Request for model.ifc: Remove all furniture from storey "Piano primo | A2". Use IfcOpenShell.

First a look at what the model holds.

```python
import ifcopenshell
import ifcopenshell.util.element

model = ifcopenshell.open("model.ifc")
print(model.schema)
storey = next(s for s in model.by_type("IfcBuildingStorey") if s.Name == "Piano primo | A2")
furniture = [e for e in ifcopenshell.util.element.get_decomposition(storey) if e.is_a("IfcFurnishingElement")]
seen = {}
for e in furniture:
    element_type = ifcopenshell.util.element.get_type(e)
    name = element_type.Name if element_type not in (None, e) else None
    seen[name] = seen.get(name, 0) + 1
for name, count in sorted(seen.items(), key=str):
    print(count, "x", name)
```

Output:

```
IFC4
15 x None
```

```python
import ifcopenshell
import ifcopenshell.api.root
import ifcopenshell.util.element

model = ifcopenshell.open("model.ifc")

storey = next(s for s in model.by_type("IfcBuildingStorey") if s.Name == "Piano primo | A2")
furniture = [e for e in ifcopenshell.util.element.get_decomposition(storey) if e.is_a("IfcFurnishingElement")]

for e in furniture:
    ifcopenshell.api.root.remove_product(model, product=e)
print(len(furniture), "removed")

model.write("model-out.ifc")
```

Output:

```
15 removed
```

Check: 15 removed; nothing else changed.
